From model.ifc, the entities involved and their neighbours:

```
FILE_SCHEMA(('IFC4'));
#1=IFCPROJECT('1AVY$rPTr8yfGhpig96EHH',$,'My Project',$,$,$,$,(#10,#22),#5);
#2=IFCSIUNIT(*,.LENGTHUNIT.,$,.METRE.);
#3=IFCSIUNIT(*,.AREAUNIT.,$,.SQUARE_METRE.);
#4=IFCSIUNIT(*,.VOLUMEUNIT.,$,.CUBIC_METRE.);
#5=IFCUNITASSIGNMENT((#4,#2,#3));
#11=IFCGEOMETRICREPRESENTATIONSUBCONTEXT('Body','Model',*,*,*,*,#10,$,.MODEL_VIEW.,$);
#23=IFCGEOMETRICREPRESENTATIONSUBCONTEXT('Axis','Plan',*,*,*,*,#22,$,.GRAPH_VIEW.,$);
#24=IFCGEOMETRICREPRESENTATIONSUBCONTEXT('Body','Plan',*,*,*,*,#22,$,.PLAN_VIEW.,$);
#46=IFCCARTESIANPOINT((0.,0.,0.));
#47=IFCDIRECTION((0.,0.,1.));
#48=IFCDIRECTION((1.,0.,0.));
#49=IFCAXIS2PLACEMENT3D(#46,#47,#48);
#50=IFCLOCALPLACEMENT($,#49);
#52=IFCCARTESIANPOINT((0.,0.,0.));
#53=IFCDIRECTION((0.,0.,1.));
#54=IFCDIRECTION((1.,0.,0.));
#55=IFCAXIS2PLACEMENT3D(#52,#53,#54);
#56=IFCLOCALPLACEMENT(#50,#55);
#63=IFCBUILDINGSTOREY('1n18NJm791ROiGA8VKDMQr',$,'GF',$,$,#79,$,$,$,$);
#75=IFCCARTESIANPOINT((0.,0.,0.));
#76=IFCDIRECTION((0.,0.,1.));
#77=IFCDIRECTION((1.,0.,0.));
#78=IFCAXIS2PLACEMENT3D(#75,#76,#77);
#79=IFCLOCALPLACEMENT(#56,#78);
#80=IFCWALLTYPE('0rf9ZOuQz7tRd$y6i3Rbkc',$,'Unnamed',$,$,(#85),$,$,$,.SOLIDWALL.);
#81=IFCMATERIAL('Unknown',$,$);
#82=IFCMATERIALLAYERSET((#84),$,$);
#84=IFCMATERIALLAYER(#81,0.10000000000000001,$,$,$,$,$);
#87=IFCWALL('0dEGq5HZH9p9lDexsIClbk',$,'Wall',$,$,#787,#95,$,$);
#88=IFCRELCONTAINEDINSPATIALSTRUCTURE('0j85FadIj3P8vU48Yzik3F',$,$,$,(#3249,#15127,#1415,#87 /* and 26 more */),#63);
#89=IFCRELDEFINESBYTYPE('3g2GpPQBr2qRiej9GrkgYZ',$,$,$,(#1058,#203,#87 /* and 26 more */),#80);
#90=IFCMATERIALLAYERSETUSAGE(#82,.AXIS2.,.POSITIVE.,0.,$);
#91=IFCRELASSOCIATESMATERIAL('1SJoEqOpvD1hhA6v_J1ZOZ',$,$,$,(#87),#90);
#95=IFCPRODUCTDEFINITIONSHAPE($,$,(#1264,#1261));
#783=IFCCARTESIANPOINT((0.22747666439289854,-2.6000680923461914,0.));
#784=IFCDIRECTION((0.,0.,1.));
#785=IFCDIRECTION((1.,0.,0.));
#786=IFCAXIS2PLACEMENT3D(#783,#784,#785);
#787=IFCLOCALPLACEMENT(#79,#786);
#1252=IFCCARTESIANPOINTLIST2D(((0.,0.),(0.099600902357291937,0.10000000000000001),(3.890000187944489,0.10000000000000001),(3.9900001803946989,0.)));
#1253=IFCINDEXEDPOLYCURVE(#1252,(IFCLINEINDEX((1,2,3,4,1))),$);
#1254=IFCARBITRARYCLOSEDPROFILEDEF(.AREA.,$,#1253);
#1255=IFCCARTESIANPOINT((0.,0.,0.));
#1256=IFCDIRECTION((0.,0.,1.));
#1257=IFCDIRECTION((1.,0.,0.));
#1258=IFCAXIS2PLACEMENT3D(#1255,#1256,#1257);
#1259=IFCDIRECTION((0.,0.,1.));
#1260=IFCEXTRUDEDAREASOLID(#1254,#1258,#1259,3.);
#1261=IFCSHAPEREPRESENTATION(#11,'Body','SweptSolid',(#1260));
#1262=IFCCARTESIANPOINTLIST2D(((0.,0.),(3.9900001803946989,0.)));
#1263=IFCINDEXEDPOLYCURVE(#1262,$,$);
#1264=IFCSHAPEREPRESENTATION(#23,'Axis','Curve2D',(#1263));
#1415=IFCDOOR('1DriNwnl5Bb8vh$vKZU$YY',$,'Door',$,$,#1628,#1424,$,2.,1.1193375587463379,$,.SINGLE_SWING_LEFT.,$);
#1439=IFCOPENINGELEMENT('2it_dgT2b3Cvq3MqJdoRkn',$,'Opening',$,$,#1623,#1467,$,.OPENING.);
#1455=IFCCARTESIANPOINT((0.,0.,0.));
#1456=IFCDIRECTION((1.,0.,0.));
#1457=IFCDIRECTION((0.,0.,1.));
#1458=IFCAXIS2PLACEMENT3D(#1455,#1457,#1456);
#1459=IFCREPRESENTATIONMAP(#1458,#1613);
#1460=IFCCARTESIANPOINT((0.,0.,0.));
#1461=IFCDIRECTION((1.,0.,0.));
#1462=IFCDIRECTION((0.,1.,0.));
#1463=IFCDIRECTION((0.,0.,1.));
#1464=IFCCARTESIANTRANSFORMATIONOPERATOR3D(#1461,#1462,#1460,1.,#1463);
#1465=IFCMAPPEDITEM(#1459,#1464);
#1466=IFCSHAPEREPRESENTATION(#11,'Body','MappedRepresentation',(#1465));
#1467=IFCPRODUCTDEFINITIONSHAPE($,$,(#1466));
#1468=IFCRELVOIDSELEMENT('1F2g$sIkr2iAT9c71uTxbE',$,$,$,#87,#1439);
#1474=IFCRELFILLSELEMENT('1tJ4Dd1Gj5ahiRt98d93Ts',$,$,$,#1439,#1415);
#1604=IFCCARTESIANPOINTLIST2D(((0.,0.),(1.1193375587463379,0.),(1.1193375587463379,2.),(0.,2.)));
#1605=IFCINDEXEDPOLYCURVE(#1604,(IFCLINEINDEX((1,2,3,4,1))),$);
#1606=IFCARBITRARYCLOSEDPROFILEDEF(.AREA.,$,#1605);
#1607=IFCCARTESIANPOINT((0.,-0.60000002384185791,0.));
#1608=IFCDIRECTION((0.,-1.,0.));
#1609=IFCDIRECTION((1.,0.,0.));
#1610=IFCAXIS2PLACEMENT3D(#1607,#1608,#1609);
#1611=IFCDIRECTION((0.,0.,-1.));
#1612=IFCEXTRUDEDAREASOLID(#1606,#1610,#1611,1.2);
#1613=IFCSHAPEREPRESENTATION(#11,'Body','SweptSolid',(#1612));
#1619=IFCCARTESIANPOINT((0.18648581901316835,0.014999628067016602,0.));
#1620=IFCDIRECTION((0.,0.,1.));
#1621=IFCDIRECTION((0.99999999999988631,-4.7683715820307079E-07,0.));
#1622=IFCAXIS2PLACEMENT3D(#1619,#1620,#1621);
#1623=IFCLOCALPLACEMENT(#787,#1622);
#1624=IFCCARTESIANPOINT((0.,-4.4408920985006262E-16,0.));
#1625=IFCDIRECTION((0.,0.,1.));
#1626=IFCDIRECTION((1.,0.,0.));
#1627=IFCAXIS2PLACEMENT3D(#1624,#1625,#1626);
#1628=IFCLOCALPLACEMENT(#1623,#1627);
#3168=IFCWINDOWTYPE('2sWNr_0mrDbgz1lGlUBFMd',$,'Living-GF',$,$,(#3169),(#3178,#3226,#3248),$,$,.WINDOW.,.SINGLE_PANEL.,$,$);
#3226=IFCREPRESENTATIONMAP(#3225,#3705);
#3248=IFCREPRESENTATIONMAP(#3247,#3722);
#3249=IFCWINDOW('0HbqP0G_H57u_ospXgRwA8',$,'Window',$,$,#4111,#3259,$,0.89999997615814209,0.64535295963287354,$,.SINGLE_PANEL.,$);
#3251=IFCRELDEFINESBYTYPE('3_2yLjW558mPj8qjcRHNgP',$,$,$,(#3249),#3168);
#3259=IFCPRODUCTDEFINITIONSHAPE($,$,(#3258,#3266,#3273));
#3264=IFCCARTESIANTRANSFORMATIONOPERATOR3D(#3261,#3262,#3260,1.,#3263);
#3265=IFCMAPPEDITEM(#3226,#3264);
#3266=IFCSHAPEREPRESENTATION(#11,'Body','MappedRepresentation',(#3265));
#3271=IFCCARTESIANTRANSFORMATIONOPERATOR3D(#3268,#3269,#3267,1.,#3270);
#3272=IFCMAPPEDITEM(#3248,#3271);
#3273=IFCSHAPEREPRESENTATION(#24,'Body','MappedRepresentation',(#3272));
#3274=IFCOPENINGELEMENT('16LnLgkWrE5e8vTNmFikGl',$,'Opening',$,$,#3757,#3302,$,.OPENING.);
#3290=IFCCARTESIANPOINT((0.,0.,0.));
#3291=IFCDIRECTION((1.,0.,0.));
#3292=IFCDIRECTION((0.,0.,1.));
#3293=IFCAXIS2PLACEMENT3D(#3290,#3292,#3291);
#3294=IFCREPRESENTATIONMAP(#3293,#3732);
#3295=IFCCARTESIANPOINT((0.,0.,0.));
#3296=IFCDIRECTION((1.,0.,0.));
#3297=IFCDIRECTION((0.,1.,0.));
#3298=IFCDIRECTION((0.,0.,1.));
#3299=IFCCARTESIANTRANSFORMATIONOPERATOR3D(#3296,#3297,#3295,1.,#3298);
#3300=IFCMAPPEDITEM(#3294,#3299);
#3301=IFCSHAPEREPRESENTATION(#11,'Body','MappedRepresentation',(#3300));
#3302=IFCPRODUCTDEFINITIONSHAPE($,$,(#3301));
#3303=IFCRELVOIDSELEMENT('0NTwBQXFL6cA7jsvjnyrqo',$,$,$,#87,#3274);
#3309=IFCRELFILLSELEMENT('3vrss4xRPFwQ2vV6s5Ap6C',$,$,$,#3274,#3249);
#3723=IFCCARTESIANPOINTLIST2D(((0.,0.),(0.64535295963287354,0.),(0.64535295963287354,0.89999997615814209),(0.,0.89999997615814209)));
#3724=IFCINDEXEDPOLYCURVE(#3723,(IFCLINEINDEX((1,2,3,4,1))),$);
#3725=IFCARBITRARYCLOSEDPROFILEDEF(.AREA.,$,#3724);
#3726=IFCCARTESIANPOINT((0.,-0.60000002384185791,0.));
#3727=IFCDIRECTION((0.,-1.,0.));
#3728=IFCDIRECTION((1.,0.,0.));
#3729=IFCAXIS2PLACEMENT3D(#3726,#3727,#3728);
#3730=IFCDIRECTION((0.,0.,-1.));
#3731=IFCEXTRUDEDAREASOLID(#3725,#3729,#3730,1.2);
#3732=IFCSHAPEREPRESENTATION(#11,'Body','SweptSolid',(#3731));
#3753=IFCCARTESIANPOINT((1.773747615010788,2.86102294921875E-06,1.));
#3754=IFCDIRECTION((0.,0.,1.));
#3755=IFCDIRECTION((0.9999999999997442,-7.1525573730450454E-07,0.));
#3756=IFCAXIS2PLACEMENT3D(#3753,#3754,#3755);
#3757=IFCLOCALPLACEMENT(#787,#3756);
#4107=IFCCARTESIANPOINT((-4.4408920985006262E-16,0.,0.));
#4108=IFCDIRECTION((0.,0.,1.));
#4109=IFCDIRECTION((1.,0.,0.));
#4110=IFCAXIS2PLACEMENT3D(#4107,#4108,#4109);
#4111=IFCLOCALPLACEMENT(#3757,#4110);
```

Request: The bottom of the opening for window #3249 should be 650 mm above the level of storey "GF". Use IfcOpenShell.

```python
import numpy as np
import ifcopenshell
import ifcopenshell.api.geometry
import ifcopenshell.geom
import ifcopenshell.util.element
import ifcopenshell.util.placement
import ifcopenshell.util.shape
import ifcopenshell.util.unit

model = ifcopenshell.open("model.ifc")
unit_scale = ifcopenshell.util.unit.calculate_unit_scale(model)

window = model.by_id(3249)
opening = window.FillsVoids[0].RelatingOpeningElement
storey = ifcopenshell.util.element.get_container(window, ifc_class="IfcBuildingStorey")
level = ifcopenshell.util.placement.get_local_placement(storey.ObjectPlacement)[2, 3]

# The opening's origin need not be at the sill, so measure its lowest point.
shape = ifcopenshell.geom.create_shape(ifcopenshell.geom.settings(), opening)
bottom = ifcopenshell.util.shape.get_shape_bottom_elevation(shape, shape.geometry) / unit_scale
dz = level + 0.65 / unit_scale - bottom

shift = np.array([0.0, 0.0, dz])
# The window is placed relative to its opening, so it follows when the opening moves.
matrix = ifcopenshell.util.placement.get_local_placement(opening.ObjectPlacement)
matrix[:3, 3] += shift
ifcopenshell.api.geometry.edit_object_placement(
    model, product=opening, matrix=matrix, is_si=False, should_transform_children=True
)

print(f"moved by {dz * unit_scale:+.3f} m")

model.write("model_updated.ifc")
```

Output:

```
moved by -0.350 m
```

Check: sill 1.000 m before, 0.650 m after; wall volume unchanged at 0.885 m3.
